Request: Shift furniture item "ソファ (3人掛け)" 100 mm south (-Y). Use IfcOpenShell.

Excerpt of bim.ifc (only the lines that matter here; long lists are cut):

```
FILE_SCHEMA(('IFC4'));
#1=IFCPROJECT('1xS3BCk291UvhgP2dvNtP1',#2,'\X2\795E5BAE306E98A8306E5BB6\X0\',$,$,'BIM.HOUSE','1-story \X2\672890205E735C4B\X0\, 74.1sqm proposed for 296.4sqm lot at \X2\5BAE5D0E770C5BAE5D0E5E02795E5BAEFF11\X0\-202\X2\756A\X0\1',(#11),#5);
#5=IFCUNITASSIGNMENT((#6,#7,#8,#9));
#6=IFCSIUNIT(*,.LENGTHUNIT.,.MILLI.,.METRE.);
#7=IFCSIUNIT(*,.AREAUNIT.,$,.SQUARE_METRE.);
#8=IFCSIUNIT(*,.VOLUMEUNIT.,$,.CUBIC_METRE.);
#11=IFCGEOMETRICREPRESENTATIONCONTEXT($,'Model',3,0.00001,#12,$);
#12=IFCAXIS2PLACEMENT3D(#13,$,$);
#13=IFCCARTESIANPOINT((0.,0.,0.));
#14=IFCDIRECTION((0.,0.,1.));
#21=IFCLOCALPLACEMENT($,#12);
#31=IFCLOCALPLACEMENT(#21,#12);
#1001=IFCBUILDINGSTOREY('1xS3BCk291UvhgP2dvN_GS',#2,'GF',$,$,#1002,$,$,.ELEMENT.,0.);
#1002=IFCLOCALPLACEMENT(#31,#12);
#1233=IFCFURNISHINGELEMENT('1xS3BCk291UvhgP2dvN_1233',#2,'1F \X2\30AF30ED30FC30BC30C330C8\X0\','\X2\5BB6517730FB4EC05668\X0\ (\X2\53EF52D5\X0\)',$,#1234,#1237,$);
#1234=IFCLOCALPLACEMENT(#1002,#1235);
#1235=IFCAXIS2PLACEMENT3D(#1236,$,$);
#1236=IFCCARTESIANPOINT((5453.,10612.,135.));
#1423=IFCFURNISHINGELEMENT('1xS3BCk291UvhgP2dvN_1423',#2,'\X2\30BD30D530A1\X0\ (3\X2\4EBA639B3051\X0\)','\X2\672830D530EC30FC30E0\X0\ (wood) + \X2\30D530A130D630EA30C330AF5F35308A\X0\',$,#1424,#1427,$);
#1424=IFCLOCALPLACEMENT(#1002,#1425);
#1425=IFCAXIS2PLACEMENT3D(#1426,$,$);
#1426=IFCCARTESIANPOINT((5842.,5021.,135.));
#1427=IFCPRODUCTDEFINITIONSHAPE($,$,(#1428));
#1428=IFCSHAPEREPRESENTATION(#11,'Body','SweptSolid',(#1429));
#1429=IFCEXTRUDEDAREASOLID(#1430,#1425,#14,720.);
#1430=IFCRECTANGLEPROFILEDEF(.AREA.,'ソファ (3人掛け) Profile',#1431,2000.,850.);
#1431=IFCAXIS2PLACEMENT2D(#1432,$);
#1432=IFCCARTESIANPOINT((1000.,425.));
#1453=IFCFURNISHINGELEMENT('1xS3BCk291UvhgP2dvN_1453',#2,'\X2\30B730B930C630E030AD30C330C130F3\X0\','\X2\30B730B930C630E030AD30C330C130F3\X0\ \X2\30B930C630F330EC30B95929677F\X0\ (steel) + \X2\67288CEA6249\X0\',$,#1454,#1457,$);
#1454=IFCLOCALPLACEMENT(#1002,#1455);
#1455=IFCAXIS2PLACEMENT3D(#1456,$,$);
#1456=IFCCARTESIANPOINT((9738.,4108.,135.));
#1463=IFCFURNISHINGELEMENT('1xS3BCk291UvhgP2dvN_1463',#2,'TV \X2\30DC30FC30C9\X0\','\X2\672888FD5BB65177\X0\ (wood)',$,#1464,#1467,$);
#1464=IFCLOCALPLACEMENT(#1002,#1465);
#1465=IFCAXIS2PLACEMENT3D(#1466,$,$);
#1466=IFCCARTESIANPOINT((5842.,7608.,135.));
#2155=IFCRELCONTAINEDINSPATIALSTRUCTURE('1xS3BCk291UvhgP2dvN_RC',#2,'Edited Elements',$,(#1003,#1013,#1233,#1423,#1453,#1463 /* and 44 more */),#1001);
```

```python
import ifcopenshell
import ifcopenshell.api.geometry
import ifcopenshell.util.placement
import ifcopenshell.util.unit

model = ifcopenshell.open("bim.ifc")
unit_scale = ifcopenshell.util.unit.calculate_unit_scale(model)

item = model.by_guid("1xS3BCk291UvhgP2dvN_1423")
matrix = ifcopenshell.util.placement.get_local_placement(item.ObjectPlacement)
matrix[1, 3] -= 0.1 / unit_scale
ifcopenshell.api.geometry.edit_object_placement(model, product=item, matrix=matrix, is_si=False)

print(ifcopenshell.util.placement.get_local_placement(item.ObjectPlacement).round(3) + 0.0)

model.write("bim_edited.ifc")
```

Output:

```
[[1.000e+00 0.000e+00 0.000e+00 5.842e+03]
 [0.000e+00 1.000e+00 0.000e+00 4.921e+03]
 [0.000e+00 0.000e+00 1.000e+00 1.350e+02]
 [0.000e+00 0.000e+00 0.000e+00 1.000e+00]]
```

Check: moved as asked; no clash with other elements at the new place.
